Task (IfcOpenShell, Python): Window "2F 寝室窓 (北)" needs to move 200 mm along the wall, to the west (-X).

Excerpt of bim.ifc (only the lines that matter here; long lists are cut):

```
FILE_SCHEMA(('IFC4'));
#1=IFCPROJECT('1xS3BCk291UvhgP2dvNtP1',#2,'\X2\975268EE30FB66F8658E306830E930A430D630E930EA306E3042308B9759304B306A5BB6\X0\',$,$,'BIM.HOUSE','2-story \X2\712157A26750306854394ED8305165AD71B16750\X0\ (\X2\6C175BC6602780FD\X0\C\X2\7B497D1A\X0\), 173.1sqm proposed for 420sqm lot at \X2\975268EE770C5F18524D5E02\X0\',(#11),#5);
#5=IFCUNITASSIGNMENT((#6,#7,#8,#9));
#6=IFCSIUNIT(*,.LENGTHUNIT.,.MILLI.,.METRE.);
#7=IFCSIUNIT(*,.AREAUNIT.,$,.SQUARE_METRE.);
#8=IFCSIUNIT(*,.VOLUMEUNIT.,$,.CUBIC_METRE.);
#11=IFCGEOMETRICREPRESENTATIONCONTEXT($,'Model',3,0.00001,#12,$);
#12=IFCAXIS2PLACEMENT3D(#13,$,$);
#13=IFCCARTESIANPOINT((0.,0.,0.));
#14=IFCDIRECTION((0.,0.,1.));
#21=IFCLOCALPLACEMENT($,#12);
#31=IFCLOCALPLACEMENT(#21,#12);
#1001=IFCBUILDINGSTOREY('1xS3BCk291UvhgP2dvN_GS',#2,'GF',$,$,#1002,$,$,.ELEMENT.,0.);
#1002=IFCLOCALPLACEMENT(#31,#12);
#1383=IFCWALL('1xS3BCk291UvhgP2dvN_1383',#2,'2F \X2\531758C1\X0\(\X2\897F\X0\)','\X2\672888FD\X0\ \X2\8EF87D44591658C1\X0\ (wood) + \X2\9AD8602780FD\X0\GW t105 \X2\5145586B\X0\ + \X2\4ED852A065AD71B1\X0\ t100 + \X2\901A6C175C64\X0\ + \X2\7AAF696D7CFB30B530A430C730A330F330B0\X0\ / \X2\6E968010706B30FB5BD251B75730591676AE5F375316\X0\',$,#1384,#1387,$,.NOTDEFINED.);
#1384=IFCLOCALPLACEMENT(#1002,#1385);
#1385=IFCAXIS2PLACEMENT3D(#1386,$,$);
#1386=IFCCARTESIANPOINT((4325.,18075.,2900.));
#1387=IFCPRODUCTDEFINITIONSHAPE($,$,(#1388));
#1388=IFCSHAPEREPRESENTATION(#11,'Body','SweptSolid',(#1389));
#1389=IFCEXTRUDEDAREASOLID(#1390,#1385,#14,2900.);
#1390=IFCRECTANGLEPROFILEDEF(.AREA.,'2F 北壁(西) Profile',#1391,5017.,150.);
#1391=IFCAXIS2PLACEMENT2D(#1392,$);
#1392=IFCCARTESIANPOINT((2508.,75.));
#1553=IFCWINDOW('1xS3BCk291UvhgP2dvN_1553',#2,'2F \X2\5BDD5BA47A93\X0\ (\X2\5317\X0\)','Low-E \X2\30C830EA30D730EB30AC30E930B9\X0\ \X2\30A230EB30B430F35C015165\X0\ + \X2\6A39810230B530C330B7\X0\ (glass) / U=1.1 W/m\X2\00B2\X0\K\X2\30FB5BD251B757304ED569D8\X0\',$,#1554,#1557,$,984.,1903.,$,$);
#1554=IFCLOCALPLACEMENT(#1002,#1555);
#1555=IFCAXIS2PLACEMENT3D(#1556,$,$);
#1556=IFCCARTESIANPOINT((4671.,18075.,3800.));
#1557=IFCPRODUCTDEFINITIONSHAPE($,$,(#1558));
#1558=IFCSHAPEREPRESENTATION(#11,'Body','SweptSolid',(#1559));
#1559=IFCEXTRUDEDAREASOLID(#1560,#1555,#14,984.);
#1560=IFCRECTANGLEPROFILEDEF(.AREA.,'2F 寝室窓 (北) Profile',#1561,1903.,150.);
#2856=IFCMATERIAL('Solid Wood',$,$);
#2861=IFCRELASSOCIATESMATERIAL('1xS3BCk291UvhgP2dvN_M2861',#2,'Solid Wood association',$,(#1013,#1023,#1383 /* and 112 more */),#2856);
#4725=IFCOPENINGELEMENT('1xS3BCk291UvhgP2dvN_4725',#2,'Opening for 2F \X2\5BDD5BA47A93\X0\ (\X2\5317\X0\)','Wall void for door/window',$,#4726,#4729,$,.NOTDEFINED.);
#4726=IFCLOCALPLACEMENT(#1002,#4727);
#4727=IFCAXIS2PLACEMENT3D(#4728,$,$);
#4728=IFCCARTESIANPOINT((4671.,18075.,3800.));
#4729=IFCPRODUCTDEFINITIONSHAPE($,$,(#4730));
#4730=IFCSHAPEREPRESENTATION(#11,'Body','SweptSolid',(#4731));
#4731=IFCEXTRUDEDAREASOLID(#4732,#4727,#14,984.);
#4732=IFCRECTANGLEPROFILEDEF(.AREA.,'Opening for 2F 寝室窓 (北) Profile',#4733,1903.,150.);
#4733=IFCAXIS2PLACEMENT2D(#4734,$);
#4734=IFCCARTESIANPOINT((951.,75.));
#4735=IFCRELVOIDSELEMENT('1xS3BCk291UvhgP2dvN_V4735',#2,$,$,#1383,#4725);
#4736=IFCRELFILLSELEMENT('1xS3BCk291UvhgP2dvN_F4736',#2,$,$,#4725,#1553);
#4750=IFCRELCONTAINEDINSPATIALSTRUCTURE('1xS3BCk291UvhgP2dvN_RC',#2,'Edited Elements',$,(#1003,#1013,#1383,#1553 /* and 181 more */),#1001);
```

```python
import ifcopenshell
import ifcopenshell.api.geometry
import ifcopenshell.util.placement
import ifcopenshell.util.unit

model = ifcopenshell.open("bim.ifc")
unit_scale = ifcopenshell.util.unit.calculate_unit_scale(model)

window = model.by_guid("1xS3BCk291UvhgP2dvN_1553")
opening = window.FillsVoids[0].RelatingOpeningElement
wall = opening.VoidsElements[0].RelatingBuildingElement

wall_matrix = ifcopenshell.util.placement.get_local_placement(wall.ObjectPlacement)
shift = wall_matrix[:3, 0] * -0.2 / unit_scale
before = ifcopenshell.util.placement.get_local_placement(window.ObjectPlacement)[:3, 3].copy()

# The window is not placed relative to its opening, so move both.
for product in (opening, window):
    matrix = ifcopenshell.util.placement.get_local_placement(product.ObjectPlacement)
    matrix[:3, 3] += shift
    ifcopenshell.api.geometry.edit_object_placement(model, product=product, matrix=matrix, is_si=False)

after = ifcopenshell.util.placement.get_local_placement(window.ObjectPlacement)[:3, 3]
print("window moved by", (after - before).round(3) + 0.0)

model.write("bim_rev.ifc")
```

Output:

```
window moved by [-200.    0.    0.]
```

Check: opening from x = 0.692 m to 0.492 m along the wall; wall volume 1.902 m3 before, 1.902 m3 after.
